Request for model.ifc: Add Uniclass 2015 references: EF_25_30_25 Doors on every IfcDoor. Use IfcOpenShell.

First a look at what the model holds.

```python
import ifcopenshell

model = ifcopenshell.open("model.ifc")
print(model.schema)
print("classifications:", [c.Name for c in model.by_type("IfcClassification")])
for ifc_class in ("IfcDoor", "IfcRoof", "IfcStair", "IfcWall", "IfcWindow"):
    print(ifc_class, len(model.by_type(ifc_class)))
```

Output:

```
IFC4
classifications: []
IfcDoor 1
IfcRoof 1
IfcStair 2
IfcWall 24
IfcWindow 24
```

```python
import ifcopenshell
import ifcopenshell.api.classification

model = ifcopenshell.open("model.ifc")

system = ifcopenshell.api.classification.add_classification(model, classification="Uniclass 2015")

codes = {
    "IfcDoor": ("EF_25_30_25", "Doors"),
}
for ifc_class, (code, name) in codes.items():
    products = model.by_type(ifc_class)
    ifcopenshell.api.classification.add_reference(
        model, products=products, classification=system, identification=code, name=name
    )
    print(code, len(products))

model.write("model_updated.ifc")
```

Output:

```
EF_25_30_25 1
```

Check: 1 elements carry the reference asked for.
